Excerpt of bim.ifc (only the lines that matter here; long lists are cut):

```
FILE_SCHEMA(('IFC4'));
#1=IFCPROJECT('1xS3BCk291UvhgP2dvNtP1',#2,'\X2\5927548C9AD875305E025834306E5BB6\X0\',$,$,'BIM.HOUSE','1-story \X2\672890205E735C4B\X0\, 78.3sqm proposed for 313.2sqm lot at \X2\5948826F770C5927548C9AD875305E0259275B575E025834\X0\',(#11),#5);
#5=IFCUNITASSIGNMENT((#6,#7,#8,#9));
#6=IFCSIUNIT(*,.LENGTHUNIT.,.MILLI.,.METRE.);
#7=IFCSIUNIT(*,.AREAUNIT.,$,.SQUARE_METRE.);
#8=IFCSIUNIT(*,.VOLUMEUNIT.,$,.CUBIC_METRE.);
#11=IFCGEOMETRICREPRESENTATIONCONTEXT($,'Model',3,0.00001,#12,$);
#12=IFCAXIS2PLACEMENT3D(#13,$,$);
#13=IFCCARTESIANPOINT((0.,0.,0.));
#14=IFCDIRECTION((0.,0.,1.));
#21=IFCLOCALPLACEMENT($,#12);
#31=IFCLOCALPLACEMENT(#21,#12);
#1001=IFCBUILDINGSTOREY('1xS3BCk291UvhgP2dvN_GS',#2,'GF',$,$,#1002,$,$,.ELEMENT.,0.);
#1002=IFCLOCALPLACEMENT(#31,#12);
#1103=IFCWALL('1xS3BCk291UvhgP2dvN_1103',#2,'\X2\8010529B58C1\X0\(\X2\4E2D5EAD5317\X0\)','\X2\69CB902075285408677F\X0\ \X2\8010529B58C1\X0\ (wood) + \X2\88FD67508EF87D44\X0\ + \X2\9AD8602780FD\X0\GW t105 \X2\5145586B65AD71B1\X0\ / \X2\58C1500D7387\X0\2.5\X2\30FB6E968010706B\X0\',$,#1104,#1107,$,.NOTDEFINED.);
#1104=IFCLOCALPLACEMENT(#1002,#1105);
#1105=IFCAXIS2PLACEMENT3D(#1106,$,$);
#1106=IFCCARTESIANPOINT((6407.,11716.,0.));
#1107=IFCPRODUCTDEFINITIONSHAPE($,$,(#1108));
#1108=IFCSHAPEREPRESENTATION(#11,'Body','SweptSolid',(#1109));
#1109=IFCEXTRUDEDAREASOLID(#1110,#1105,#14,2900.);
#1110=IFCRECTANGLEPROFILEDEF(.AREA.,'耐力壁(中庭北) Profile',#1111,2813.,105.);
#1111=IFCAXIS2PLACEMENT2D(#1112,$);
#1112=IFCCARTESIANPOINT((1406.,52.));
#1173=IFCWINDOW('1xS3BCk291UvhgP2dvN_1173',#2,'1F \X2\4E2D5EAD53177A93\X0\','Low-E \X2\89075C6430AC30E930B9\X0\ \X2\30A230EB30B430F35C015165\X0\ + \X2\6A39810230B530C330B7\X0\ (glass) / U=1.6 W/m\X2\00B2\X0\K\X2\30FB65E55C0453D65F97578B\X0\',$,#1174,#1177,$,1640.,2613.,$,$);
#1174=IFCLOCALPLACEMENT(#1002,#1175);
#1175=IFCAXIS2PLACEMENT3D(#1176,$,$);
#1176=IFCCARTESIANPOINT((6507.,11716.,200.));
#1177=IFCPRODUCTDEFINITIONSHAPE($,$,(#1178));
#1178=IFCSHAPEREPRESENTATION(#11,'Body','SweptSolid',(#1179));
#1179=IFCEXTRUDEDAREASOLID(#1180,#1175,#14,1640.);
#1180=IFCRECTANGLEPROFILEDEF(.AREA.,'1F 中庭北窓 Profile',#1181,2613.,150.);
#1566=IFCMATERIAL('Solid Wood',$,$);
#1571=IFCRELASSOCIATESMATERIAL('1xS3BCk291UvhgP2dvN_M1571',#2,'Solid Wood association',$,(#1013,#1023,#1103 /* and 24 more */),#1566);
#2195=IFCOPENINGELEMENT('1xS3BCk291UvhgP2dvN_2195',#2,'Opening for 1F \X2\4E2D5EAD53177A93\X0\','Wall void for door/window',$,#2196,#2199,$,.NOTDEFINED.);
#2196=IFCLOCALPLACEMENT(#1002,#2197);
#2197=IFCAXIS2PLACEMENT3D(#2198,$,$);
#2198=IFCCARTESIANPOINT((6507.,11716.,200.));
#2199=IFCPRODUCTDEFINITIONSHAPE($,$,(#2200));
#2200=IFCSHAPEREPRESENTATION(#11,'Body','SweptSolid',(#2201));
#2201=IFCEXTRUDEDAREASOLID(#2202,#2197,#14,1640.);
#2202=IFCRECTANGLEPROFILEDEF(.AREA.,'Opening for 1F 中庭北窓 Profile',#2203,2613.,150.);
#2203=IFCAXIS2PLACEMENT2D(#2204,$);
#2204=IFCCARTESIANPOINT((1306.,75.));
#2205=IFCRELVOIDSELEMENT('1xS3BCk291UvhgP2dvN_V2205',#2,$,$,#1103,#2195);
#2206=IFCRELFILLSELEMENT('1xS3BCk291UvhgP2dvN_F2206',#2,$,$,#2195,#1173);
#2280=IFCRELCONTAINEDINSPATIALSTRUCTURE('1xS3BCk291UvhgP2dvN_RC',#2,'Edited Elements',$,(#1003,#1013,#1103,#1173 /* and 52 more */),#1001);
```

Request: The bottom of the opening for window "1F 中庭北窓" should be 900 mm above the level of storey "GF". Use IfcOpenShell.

```python
import numpy as np
import ifcopenshell
import ifcopenshell.api.geometry
import ifcopenshell.geom
import ifcopenshell.util.element
import ifcopenshell.util.placement
import ifcopenshell.util.shape
import ifcopenshell.util.unit

model = ifcopenshell.open("bim.ifc")
unit_scale = ifcopenshell.util.unit.calculate_unit_scale(model)

window = model.by_id(1173)
opening = window.FillsVoids[0].RelatingOpeningElement
storey = ifcopenshell.util.element.get_container(window, ifc_class="IfcBuildingStorey")
level = ifcopenshell.util.placement.get_local_placement(storey.ObjectPlacement)[2, 3]

# The opening's origin need not be at the sill, so measure its lowest point.
shape = ifcopenshell.geom.create_shape(ifcopenshell.geom.settings(), opening)
bottom = ifcopenshell.util.shape.get_shape_bottom_elevation(shape, shape.geometry) / unit_scale
dz = level + 0.9 / unit_scale - bottom

shift = np.array([0.0, 0.0, dz])
# The window is not placed relative to its opening, so move both.
for product in (opening, window):
    matrix = ifcopenshell.util.placement.get_local_placement(product.ObjectPlacement)
    matrix[:3, 3] += shift
    ifcopenshell.api.geometry.edit_object_placement(model, product=product, matrix=matrix, is_si=False)

print(f"moved by {dz * unit_scale:+.3f} m")

model.write("bim-out.ifc")
```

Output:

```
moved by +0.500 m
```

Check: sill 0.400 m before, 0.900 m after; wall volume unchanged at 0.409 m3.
